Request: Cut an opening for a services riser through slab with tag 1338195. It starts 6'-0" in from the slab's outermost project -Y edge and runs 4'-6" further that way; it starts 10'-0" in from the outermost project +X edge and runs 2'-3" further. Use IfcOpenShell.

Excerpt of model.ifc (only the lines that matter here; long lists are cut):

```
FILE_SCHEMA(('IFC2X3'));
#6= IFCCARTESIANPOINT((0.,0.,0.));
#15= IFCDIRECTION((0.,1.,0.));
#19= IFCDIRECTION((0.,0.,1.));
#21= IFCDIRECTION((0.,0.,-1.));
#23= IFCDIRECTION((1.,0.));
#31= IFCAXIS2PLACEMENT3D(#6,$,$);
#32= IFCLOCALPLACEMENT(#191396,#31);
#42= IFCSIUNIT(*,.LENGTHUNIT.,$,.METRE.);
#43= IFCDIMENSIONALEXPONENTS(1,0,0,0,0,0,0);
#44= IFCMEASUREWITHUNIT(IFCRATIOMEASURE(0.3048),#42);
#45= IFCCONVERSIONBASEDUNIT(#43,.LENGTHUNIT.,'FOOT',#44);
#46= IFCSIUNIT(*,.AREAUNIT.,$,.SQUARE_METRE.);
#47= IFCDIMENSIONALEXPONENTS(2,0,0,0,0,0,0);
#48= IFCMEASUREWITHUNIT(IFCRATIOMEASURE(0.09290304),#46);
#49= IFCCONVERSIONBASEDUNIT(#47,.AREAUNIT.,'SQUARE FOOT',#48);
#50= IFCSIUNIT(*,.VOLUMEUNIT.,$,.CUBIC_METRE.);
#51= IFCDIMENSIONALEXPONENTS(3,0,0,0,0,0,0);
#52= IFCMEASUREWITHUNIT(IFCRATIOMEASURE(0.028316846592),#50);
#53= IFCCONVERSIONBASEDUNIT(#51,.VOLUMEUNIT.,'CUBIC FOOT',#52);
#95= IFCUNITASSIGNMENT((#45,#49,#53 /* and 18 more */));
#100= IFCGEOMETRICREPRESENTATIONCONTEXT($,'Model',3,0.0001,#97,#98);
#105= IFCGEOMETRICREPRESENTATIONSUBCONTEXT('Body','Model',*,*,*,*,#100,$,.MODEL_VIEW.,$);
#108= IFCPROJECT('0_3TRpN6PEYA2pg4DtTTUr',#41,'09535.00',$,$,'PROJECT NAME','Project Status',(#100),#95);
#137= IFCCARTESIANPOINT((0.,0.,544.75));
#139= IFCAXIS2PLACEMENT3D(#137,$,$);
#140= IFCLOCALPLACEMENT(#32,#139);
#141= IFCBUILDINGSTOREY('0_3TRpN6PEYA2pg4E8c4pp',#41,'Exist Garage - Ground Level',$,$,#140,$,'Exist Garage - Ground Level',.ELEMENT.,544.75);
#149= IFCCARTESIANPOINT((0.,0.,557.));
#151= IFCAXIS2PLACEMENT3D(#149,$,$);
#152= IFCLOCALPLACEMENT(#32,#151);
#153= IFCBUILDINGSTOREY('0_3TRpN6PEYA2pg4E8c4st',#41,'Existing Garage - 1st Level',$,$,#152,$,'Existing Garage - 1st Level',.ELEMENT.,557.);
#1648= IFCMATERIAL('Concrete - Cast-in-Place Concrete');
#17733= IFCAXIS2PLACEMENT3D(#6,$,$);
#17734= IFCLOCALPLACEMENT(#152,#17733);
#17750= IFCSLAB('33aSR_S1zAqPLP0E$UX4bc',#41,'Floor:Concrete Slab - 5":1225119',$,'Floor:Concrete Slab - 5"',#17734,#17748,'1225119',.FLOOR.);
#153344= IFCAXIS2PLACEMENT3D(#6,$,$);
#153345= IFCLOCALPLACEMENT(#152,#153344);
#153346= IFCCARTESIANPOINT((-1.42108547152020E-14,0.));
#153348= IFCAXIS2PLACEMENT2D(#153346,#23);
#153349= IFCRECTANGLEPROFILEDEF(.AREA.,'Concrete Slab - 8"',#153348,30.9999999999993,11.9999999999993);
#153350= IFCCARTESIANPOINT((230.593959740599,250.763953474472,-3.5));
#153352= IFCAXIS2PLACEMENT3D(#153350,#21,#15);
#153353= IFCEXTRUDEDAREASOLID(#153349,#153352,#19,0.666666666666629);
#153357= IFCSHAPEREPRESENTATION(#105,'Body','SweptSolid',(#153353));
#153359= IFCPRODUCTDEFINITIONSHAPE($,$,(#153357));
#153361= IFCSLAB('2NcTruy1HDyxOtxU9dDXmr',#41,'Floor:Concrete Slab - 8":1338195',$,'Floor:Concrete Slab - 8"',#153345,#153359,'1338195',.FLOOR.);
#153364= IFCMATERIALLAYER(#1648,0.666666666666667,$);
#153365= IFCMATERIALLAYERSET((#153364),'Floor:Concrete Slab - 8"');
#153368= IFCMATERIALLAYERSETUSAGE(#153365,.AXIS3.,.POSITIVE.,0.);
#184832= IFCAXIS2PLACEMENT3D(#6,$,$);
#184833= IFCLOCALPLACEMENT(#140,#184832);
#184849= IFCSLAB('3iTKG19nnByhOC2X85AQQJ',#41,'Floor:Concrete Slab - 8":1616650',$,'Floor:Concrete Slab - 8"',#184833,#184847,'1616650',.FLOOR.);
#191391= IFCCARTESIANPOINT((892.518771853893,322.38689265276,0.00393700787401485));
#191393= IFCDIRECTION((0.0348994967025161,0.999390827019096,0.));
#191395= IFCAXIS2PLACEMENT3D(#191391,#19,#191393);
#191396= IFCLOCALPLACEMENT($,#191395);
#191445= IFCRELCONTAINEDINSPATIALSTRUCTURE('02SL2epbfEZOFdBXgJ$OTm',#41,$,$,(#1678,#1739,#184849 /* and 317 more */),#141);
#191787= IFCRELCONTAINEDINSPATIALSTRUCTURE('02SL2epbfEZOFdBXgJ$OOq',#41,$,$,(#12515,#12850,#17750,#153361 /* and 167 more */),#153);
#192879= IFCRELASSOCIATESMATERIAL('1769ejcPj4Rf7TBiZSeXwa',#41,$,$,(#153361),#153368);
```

```python
import numpy as np
import ifcopenshell
import ifcopenshell.api.feature
import ifcopenshell.api.geometry
import ifcopenshell.api.root
import ifcopenshell.geom
import ifcopenshell.util.placement
import ifcopenshell.util.representation
import ifcopenshell.util.shape
import ifcopenshell.util.unit

model = ifcopenshell.open("model.ifc")
unit_scale = ifcopenshell.util.unit.calculate_unit_scale(model)
settings = ifcopenshell.geom.settings()


def volume(element):
    """Net volume in cubic metres, openings subtracted."""
    shape = ifcopenshell.geom.create_shape(settings, element)
    return ifcopenshell.util.shape.get_volume(shape.geometry)


slab = model.by_guid("2NcTruy1HDyxOtxU9dDXmr")
before = volume(slab)

# Extent in the slab's own axes, in metres. The edges named are its -X and -Y sides.
slab_shape = ifcopenshell.geom.create_shape(settings, slab)
vertices = ifcopenshell.util.shape.get_vertices(slab_shape.geometry)
x_min, y_min, bottom = vertices.min(axis=0)
top = vertices[:, 2].max()

opening = ifcopenshell.api.root.create_entity(model, ifc_class="IfcOpeningElement", name="Services riser opening")
context = ifcopenshell.util.representation.get_context(model, "Model", "Body", "MODEL_VIEW")
width, depth = 1.3716, 0.6858
outline = [(0.0, 0.0), (width, 0.0), (width, depth), (0.0, depth), (0.0, 0.0)]
# Overshoot both faces by 50 mm so the cut is clean.
shape = ifcopenshell.api.geometry.add_slab_representation(
    model, context=context, depth=top - bottom + 0.1, polyline=outline
)
ifcopenshell.api.geometry.assign_representation(model, product=opening, representation=shape)

matrix = ifcopenshell.util.placement.get_local_placement(slab.ObjectPlacement)
matrix[:, 3] = matrix @ np.append(np.array([x_min + 1.8288, y_min + 3.048, bottom - 0.05]) / unit_scale, 1.0)
ifcopenshell.api.geometry.edit_object_placement(model, product=opening, matrix=matrix, is_si=False)
ifcopenshell.api.feature.add_feature(model, feature=opening, element=slab)

after = volume(slab)

print(f"slab volume {before:.3f} -> {after:.3f} m3")

model.write("model_rev.ifc")
```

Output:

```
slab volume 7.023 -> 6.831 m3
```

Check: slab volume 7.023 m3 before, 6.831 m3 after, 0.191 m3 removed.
